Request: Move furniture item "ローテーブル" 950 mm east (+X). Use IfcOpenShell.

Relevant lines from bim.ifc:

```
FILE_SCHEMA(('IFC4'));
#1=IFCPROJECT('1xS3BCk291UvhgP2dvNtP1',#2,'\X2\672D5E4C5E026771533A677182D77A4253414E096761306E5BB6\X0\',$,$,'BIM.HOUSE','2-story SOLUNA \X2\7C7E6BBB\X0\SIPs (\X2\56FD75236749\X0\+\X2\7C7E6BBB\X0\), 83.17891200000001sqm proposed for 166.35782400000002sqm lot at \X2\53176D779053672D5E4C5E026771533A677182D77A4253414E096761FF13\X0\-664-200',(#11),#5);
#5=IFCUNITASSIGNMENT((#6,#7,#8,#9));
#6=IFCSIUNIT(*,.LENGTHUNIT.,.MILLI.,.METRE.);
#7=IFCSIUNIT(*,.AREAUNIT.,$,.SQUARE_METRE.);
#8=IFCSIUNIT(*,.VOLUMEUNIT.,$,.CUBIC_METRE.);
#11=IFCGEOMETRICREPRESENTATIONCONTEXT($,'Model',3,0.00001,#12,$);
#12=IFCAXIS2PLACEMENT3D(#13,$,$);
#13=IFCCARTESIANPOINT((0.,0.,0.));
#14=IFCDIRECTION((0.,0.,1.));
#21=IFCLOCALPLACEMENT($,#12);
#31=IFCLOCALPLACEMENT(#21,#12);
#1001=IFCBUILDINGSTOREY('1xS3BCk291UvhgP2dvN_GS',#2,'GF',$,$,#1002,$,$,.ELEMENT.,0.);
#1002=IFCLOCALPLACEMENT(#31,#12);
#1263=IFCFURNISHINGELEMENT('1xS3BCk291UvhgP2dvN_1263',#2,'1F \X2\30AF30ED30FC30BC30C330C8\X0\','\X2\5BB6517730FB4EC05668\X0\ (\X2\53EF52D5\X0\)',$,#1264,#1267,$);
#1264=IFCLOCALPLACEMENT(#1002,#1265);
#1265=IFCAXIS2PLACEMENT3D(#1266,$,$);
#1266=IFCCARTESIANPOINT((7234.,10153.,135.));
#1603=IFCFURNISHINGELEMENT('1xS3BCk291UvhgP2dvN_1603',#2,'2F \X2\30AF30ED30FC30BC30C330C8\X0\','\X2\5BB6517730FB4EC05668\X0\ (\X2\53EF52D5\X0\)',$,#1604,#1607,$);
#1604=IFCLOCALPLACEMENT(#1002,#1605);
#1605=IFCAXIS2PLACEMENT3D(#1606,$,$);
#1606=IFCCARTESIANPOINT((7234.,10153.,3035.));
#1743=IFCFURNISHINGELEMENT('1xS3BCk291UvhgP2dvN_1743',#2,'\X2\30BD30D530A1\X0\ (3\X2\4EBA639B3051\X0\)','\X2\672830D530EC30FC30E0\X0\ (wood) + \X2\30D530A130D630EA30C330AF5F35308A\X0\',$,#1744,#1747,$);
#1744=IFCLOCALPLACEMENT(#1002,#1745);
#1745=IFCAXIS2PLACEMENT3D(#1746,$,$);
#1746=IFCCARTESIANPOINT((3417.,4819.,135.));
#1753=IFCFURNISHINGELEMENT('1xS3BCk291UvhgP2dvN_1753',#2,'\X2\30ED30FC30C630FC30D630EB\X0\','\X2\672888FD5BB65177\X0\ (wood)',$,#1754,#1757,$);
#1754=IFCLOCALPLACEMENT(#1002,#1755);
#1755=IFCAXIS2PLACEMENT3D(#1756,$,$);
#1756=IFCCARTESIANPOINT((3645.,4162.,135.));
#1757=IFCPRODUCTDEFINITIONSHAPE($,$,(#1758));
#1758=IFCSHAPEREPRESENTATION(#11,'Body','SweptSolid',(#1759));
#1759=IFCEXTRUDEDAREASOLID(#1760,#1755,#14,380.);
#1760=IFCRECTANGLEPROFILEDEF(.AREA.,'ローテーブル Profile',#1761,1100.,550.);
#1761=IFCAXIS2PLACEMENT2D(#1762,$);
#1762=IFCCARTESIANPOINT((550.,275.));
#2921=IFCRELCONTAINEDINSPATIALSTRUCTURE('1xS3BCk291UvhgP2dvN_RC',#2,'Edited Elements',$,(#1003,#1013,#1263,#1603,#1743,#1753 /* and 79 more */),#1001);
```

```python
import ifcopenshell
import ifcopenshell.api.geometry
import ifcopenshell.util.placement
import ifcopenshell.util.unit

model = ifcopenshell.open("bim.ifc")
unit_scale = ifcopenshell.util.unit.calculate_unit_scale(model)

item = model.by_id(1753)
matrix = ifcopenshell.util.placement.get_local_placement(item.ObjectPlacement)
matrix[0, 3] += 0.95 / unit_scale
ifcopenshell.api.geometry.edit_object_placement(model, product=item, matrix=matrix, is_si=False)

print(ifcopenshell.util.placement.get_local_placement(item.ObjectPlacement).round(3) + 0.0)

model.write("bim-out.ifc")
```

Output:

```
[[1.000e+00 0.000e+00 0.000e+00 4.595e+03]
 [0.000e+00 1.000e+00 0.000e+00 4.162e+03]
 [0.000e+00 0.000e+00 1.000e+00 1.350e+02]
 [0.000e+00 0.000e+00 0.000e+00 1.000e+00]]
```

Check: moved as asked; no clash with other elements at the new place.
